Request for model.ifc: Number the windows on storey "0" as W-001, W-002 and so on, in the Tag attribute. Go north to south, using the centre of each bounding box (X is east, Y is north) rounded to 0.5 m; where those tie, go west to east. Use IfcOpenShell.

First a look at what the model holds.

```python
import ifcopenshell
import ifcopenshell.util.element
import ifcopenshell.util.placement

model = ifcopenshell.open("model.ifc")
print(model.schema)
storey = next(s for s in model.by_type("IfcBuildingStorey") if s.Name == "0")
windows = [e for e in ifcopenshell.util.element.get_decomposition(storey) if e.is_a("IfcWindow")]
for e in sorted(windows, key=lambda e: e.id()):
    origin = ifcopenshell.util.placement.get_local_placement(e.ObjectPlacement)[:3, 3]
    print(e.id(), e.Tag, e.Name, origin.round(2) + 0.0, sep=" | ")
```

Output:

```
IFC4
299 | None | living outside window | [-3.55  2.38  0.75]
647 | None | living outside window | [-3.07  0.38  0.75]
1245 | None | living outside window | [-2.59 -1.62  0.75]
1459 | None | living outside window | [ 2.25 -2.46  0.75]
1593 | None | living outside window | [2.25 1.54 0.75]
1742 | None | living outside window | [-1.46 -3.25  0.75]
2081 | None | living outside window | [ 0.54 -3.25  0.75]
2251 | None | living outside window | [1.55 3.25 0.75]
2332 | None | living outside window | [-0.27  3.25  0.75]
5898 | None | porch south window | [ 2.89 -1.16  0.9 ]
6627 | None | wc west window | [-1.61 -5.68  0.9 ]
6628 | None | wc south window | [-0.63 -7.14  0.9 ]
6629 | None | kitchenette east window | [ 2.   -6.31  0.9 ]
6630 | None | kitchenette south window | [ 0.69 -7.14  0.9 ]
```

```python
import ifcopenshell
import ifcopenshell.geom
import ifcopenshell.util.element
import ifcopenshell.util.shape

model = ifcopenshell.open("model.ifc")
settings = ifcopenshell.geom.settings()
settings.set("use-world-coords", True)


def centre(element):
    shape = ifcopenshell.geom.create_shape(settings, element)
    return ifcopenshell.util.shape.get_bbox_centroid(shape.geometry)


storey = next(s for s in model.by_type("IfcBuildingStorey") if s.Name == "0")
windows = [e for e in ifcopenshell.util.element.get_decomposition(storey) if e.is_a("IfcWindow")]

# Insertion points can sit at a corner or the storey origin, so sort by the geometry (in metres).
centres = {e: centre(e) for e in windows}
windows.sort(key=lambda e: (-round(centres[e][1] / 0.5), centres[e][0]))

for i, e in enumerate(windows, start=1):
    number = f"W-0{i:02d}"
    e.Tag = number
    print(e.id(), number)

model.write("model_updated.ifc")
```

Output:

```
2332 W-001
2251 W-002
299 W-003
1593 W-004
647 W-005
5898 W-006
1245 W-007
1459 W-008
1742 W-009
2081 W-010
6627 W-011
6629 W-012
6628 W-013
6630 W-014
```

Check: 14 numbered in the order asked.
